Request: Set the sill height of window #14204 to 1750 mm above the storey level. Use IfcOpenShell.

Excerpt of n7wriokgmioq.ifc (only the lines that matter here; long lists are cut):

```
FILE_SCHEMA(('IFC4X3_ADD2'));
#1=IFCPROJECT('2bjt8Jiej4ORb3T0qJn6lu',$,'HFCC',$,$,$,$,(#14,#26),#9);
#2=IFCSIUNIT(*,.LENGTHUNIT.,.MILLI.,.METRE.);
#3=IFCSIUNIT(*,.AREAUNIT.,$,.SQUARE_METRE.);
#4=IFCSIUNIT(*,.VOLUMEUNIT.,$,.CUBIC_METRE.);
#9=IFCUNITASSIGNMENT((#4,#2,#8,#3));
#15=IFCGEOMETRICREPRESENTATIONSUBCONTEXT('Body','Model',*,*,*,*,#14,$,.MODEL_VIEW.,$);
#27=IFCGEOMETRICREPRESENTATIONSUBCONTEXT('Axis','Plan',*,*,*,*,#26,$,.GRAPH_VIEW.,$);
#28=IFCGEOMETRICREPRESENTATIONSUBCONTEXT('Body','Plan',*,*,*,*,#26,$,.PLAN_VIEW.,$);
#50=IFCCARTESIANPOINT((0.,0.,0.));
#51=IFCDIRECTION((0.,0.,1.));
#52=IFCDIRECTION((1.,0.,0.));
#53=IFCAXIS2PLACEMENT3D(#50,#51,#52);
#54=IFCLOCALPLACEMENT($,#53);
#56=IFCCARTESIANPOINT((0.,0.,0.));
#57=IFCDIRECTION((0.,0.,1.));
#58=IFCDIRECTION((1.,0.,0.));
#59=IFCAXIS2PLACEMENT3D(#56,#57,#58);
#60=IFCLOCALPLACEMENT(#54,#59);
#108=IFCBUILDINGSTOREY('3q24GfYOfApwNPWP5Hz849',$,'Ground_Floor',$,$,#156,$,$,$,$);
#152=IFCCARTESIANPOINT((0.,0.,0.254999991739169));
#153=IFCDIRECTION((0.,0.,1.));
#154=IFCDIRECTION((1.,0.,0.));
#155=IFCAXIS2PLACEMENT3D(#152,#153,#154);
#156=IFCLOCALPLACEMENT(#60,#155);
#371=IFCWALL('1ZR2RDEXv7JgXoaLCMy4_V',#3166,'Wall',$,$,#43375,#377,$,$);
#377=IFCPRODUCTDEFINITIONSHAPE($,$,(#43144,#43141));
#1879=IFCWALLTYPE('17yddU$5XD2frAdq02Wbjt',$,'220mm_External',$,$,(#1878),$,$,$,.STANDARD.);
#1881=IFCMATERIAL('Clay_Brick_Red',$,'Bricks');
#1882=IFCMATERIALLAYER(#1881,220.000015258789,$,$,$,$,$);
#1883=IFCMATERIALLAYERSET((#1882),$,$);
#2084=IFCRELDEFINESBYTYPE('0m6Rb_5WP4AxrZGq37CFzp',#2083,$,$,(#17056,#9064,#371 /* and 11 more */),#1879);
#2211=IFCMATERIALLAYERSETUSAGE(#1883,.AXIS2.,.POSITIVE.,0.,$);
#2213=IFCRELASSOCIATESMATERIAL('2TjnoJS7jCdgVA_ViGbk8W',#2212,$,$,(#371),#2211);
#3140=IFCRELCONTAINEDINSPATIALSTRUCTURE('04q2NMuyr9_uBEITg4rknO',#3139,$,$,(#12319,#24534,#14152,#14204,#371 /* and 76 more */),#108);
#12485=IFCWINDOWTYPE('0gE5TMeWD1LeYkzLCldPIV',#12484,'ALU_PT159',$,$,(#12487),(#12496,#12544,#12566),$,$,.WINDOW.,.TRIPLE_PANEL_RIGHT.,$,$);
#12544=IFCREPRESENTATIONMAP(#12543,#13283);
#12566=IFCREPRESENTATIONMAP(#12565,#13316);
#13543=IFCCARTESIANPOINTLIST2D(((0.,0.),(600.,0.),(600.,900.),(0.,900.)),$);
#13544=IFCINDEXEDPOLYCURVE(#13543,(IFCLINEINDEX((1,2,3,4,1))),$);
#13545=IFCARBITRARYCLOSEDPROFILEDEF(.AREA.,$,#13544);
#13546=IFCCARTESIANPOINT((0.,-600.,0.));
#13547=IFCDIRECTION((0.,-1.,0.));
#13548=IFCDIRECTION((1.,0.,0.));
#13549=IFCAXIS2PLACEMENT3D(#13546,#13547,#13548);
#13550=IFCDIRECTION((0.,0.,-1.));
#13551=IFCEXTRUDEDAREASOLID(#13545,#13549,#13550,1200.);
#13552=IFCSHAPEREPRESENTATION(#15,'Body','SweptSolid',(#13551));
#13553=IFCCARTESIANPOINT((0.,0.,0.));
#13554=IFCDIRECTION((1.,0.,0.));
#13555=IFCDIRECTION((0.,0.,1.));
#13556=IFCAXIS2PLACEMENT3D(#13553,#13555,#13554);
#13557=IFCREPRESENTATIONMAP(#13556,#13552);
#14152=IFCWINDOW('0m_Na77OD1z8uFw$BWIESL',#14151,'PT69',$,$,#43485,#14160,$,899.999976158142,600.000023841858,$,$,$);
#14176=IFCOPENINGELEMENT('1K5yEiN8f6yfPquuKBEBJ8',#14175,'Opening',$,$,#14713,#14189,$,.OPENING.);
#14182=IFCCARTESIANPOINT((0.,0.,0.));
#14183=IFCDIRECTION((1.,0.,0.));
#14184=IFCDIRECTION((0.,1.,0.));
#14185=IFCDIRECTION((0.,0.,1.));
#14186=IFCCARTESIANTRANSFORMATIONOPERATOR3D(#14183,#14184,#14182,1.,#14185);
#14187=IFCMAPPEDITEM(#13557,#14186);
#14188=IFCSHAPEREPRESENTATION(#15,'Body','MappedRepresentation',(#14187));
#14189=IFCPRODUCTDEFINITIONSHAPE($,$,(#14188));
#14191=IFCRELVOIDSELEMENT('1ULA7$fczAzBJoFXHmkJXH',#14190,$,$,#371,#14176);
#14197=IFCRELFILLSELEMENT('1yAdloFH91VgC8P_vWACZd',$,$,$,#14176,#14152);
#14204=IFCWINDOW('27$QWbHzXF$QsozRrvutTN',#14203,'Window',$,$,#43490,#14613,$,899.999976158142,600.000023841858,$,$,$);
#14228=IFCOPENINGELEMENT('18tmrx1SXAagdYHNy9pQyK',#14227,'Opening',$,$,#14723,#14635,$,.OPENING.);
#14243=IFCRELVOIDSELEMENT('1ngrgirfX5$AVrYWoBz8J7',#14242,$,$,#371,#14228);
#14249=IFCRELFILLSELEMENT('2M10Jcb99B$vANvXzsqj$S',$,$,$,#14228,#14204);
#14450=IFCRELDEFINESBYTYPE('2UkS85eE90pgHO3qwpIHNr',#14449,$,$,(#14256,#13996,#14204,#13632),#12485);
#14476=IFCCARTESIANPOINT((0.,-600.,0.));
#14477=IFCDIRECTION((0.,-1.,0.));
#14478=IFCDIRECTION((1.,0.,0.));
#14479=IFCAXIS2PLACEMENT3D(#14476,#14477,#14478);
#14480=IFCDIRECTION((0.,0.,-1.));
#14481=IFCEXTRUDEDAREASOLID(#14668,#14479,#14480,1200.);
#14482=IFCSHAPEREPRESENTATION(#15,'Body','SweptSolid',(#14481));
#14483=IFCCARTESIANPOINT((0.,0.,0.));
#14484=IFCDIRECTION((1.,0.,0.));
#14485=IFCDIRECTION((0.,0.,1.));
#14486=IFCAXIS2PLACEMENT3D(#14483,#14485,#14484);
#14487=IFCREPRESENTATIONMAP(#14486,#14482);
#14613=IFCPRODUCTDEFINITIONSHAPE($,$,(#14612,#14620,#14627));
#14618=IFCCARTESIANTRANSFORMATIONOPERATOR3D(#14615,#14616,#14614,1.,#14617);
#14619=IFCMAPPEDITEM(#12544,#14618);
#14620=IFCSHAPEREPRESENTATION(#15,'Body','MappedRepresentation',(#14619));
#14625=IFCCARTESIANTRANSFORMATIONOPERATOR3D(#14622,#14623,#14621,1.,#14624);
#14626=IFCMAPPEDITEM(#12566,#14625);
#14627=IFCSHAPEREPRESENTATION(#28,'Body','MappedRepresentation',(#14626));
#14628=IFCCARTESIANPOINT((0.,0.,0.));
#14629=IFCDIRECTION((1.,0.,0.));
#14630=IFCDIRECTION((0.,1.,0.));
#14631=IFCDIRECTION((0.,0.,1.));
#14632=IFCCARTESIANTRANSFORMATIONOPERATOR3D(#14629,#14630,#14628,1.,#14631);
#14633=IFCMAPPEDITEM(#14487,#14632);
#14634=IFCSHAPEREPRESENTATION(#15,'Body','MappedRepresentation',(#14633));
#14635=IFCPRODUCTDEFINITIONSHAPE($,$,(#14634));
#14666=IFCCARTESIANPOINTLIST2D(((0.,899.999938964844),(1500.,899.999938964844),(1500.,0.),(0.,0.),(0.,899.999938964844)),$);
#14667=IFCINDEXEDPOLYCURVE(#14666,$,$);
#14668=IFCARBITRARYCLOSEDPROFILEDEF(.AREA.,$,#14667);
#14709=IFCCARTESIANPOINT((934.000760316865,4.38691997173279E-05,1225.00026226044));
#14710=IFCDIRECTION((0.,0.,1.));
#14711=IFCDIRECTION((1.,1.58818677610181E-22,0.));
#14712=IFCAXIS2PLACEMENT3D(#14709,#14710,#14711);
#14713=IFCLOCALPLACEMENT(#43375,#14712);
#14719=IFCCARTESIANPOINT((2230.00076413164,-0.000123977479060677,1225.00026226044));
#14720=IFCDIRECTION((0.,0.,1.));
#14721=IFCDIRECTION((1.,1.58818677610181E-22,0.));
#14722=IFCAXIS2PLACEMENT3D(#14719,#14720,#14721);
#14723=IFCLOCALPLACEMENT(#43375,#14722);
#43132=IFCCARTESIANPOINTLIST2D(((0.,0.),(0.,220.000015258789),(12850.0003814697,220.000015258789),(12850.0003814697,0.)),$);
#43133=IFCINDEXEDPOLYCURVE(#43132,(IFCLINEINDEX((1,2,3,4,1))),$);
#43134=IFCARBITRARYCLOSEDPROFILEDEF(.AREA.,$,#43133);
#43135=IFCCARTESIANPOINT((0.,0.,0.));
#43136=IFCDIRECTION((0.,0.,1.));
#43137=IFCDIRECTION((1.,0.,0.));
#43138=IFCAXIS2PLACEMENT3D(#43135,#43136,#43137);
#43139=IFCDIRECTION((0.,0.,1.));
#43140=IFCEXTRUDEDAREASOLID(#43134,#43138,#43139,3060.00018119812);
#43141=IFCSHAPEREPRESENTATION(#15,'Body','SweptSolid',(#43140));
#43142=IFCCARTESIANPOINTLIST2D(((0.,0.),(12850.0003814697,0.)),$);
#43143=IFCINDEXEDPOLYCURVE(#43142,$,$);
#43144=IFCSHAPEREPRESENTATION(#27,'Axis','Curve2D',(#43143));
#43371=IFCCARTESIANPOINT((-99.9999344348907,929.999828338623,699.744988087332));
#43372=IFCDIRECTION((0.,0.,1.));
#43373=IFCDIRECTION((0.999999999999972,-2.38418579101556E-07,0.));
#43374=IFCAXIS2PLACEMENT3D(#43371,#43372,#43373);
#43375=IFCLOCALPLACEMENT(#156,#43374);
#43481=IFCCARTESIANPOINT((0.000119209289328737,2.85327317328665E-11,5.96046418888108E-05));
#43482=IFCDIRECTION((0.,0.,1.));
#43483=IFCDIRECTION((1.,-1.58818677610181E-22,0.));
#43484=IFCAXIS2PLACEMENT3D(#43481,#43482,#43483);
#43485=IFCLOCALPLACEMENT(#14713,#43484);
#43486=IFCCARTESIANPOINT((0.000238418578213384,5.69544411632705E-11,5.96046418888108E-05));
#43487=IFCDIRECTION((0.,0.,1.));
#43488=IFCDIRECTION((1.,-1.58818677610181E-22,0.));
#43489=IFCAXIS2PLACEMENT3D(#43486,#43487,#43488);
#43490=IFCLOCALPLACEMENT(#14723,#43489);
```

```python
import numpy as np
import ifcopenshell
import ifcopenshell.api.geometry
import ifcopenshell.geom
import ifcopenshell.util.element
import ifcopenshell.util.placement
import ifcopenshell.util.shape
import ifcopenshell.util.unit

model = ifcopenshell.open("n7wriokgmioq.ifc")
unit_scale = ifcopenshell.util.unit.calculate_unit_scale(model)

window = model.by_guid("27$QWbHzXF$QsozRrvutTN")
opening = window.FillsVoids[0].RelatingOpeningElement
storey = ifcopenshell.util.element.get_container(window, ifc_class="IfcBuildingStorey")
level = ifcopenshell.util.placement.get_local_placement(storey.ObjectPlacement)[2, 3]

# The opening's origin need not be at the sill, so measure its lowest point.
shape = ifcopenshell.geom.create_shape(ifcopenshell.geom.settings(), opening)
bottom = ifcopenshell.util.shape.get_shape_bottom_elevation(shape, shape.geometry) / unit_scale
dz = level + 1.75 / unit_scale - bottom

shift = np.array([0.0, 0.0, dz])
# The window is placed relative to its opening, so it follows when the opening moves.
matrix = ifcopenshell.util.placement.get_local_placement(opening.ObjectPlacement)
matrix[:3, 3] += shift
ifcopenshell.api.geometry.edit_object_placement(
    model, product=opening, matrix=matrix, is_si=False, should_transform_children=True
)

print(f"moved by {dz * unit_scale:+.3f} m")

model.write("n7wriokgmioq_rev.ifc")
```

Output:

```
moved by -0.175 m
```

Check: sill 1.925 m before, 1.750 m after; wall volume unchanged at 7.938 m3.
